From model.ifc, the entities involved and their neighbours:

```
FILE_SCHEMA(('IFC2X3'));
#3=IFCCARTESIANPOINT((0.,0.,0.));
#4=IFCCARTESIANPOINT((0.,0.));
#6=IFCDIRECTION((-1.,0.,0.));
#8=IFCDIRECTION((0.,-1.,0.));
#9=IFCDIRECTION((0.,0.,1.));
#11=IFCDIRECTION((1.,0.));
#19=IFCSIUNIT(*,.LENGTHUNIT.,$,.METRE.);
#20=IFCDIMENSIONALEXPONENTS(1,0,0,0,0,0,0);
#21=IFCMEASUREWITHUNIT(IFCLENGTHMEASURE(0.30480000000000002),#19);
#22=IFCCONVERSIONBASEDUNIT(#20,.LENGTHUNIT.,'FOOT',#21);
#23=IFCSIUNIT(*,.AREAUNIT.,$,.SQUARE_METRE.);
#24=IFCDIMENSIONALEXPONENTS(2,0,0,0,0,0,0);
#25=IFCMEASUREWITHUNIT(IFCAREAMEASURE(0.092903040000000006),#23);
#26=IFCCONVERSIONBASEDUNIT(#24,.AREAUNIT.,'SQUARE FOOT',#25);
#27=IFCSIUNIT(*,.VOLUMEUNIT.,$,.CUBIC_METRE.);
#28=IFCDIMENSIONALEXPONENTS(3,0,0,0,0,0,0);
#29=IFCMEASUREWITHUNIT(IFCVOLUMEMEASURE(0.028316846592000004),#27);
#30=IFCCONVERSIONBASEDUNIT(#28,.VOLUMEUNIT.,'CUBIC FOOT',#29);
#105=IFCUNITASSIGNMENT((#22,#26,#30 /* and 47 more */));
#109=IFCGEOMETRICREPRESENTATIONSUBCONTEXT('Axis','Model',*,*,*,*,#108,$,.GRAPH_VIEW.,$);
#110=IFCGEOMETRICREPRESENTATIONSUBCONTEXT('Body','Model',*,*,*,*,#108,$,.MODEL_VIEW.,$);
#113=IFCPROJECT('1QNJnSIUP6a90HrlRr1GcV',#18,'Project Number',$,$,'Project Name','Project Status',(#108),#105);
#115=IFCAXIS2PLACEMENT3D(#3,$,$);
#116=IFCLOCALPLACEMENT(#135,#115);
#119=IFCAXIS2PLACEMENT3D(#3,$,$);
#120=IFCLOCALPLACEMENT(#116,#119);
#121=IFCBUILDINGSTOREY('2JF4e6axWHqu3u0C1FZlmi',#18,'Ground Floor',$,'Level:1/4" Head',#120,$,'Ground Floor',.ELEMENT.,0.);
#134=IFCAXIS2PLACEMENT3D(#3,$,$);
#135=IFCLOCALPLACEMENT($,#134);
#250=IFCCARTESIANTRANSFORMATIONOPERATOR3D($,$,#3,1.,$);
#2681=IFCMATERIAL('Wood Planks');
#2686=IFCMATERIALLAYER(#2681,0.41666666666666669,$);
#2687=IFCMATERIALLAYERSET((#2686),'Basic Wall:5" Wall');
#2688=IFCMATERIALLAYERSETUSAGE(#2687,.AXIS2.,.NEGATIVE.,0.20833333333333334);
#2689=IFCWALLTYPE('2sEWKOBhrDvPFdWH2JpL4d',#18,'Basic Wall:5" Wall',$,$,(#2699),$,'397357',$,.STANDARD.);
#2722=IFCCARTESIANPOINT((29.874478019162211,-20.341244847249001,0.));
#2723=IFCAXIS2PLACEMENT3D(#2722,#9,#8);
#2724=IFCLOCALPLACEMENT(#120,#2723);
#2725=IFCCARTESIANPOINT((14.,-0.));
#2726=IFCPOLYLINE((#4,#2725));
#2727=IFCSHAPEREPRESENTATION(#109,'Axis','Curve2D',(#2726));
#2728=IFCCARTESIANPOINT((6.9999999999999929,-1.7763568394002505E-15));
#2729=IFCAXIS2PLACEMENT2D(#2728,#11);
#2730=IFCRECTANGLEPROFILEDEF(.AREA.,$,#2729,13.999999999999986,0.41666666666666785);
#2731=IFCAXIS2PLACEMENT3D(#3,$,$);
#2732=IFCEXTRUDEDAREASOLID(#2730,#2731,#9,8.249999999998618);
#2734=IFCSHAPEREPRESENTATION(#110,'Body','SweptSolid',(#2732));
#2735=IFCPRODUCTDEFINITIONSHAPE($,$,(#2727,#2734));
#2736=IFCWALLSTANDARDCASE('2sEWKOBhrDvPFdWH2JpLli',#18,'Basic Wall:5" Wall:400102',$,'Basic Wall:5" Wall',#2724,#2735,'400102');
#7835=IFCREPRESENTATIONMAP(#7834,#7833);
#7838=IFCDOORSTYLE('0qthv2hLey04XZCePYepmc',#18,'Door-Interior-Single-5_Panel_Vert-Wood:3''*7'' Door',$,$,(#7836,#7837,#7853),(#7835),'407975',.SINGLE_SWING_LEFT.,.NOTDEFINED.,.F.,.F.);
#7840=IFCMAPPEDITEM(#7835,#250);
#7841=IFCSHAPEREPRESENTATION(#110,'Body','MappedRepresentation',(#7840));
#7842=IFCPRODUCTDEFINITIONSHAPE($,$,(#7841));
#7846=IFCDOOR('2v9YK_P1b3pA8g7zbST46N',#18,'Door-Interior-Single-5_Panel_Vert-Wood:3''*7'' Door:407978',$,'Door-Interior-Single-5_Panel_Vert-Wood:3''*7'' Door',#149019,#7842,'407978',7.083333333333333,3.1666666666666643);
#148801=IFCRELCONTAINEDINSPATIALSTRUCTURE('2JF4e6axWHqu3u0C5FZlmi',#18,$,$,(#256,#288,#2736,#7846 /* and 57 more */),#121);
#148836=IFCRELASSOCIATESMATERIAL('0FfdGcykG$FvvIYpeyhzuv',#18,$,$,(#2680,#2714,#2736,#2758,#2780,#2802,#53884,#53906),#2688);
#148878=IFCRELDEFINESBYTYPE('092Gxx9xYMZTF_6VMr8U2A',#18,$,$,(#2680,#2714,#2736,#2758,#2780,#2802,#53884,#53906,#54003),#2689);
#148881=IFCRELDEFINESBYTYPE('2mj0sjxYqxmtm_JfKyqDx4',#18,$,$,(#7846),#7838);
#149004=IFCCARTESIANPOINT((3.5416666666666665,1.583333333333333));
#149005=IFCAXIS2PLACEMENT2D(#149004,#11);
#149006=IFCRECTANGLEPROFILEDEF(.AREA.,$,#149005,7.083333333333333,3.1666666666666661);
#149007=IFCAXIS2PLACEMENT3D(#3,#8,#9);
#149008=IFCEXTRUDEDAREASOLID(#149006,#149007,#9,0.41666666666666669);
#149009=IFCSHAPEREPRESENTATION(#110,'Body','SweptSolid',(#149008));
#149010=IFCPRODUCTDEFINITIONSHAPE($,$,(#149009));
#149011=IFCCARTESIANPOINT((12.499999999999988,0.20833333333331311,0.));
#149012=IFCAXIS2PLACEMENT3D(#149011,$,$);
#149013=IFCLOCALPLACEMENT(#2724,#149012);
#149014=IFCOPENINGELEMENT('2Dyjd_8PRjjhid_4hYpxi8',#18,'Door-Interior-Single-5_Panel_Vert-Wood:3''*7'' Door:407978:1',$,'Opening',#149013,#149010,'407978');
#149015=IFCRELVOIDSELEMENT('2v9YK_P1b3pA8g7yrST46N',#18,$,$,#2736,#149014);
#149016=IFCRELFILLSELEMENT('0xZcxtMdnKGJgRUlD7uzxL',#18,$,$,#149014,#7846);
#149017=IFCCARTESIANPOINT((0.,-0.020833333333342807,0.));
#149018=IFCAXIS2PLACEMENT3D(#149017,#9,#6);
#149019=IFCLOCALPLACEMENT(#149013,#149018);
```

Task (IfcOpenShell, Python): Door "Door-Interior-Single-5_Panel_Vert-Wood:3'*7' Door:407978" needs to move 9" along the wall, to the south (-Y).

```python
import ifcopenshell
import ifcopenshell.api.geometry
import ifcopenshell.util.placement
import ifcopenshell.util.unit

model = ifcopenshell.open("model.ifc")
unit_scale = ifcopenshell.util.unit.calculate_unit_scale(model)

door = model.by_id(7846)
opening = door.FillsVoids[0].RelatingOpeningElement
wall = opening.VoidsElements[0].RelatingBuildingElement

wall_matrix = ifcopenshell.util.placement.get_local_placement(wall.ObjectPlacement)
shift = wall_matrix[:3, 0] * 9 * 0.0254 / unit_scale
before = ifcopenshell.util.placement.get_local_placement(door.ObjectPlacement)[:3, 3].copy()

# The door is placed relative to its opening, so it follows when the opening moves.
matrix = ifcopenshell.util.placement.get_local_placement(opening.ObjectPlacement)
matrix[:3, 3] += shift
ifcopenshell.api.geometry.edit_object_placement(
    model, product=opening, matrix=matrix, is_si=False, should_transform_children=True
)

after = ifcopenshell.util.placement.get_local_placement(door.ObjectPlacement)[:3, 3]
print("door moved by", (after - before).round(3) + 0.0)

model.write("model_rev.ifc")
```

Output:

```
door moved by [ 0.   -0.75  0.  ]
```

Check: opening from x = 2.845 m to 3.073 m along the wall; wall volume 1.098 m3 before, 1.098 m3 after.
